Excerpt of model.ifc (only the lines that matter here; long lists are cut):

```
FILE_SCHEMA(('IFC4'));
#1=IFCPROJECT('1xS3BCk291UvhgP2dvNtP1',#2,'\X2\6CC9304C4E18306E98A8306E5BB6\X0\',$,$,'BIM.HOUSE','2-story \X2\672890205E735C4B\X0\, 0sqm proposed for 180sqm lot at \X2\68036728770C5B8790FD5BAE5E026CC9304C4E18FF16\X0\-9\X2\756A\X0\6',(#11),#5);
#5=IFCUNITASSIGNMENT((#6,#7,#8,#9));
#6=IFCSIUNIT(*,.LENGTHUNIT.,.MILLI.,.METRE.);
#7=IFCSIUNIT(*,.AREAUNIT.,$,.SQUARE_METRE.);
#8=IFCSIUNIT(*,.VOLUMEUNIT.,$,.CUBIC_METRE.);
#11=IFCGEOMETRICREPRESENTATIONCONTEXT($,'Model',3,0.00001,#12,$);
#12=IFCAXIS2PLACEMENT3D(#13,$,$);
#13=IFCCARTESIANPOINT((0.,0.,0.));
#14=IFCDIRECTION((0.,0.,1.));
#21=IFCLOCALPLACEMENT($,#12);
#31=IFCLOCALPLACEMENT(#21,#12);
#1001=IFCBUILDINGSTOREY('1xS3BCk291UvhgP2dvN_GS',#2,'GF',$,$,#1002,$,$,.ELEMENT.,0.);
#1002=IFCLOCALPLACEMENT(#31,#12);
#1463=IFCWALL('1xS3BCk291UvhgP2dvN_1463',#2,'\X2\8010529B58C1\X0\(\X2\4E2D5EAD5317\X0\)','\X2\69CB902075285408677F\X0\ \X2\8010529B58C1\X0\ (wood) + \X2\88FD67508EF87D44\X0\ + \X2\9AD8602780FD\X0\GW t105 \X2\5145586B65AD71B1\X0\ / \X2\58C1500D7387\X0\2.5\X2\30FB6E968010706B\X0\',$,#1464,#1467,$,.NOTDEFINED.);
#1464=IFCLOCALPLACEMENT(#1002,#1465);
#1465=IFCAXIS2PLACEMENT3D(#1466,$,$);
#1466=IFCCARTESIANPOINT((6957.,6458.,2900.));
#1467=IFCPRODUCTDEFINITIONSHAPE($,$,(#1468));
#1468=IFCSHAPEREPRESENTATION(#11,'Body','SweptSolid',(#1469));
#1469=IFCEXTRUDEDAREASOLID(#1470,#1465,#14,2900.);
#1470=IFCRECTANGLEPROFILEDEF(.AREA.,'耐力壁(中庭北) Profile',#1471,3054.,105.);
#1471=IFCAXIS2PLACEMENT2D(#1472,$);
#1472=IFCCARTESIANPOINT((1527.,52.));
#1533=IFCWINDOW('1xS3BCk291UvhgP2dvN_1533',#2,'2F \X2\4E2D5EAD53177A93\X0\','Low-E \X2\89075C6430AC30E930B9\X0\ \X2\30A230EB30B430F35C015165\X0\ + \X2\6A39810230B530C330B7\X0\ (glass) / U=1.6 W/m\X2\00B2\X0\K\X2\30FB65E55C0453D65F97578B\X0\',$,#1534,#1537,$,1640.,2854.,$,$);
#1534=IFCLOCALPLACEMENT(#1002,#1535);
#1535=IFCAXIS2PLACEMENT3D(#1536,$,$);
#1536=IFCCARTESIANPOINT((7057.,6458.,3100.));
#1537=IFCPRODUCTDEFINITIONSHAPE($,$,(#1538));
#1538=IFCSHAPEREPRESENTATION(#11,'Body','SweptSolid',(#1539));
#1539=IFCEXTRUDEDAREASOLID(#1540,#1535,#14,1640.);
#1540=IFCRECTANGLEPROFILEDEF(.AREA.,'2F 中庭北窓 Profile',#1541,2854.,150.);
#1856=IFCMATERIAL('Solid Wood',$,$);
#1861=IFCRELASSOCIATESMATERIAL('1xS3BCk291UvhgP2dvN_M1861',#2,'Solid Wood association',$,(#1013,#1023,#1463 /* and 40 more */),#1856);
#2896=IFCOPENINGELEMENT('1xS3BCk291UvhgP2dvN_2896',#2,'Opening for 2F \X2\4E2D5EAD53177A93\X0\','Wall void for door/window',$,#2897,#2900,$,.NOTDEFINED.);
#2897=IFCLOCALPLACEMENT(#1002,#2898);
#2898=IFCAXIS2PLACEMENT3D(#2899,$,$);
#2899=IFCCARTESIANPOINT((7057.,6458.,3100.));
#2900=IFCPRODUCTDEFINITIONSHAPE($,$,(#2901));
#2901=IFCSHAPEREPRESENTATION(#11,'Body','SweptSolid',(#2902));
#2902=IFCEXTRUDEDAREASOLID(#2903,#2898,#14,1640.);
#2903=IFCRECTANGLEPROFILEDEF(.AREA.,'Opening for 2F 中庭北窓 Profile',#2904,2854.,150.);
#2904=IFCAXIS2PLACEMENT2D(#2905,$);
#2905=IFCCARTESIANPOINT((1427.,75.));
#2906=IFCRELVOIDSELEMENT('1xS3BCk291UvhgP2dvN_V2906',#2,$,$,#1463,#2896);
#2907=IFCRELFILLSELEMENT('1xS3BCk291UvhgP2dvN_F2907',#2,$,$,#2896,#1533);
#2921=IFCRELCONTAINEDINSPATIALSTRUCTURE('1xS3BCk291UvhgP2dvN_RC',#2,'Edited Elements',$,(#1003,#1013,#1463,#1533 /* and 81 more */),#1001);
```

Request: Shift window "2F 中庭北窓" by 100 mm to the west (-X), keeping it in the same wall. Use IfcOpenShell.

```python
import ifcopenshell
import ifcopenshell.api.geometry
import ifcopenshell.util.placement

model = ifcopenshell.open("model.ifc")

window = model.by_guid("1xS3BCk291UvhgP2dvN_1533")
opening = window.FillsVoids[0].RelatingOpeningElement
wall = opening.VoidsElements[0].RelatingBuildingElement

wall_matrix = ifcopenshell.util.placement.get_local_placement(wall.ObjectPlacement)
shift = wall_matrix[:3, 0] * -100.0
before = ifcopenshell.util.placement.get_local_placement(window.ObjectPlacement)[:3, 3].copy()

# The window is not placed relative to its opening, so move both.
for product in (opening, window):
    matrix = ifcopenshell.util.placement.get_local_placement(product.ObjectPlacement)
    matrix[:3, 3] += shift
    ifcopenshell.api.geometry.edit_object_placement(model, product=product, matrix=matrix, is_si=False)

after = ifcopenshell.util.placement.get_local_placement(window.ObjectPlacement)[:3, 3]
print("window moved by", (after - before).round(3) + 0.0)

model.write("model_updated.ifc")
```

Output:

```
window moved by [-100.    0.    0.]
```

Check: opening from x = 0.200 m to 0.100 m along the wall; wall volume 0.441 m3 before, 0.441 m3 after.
